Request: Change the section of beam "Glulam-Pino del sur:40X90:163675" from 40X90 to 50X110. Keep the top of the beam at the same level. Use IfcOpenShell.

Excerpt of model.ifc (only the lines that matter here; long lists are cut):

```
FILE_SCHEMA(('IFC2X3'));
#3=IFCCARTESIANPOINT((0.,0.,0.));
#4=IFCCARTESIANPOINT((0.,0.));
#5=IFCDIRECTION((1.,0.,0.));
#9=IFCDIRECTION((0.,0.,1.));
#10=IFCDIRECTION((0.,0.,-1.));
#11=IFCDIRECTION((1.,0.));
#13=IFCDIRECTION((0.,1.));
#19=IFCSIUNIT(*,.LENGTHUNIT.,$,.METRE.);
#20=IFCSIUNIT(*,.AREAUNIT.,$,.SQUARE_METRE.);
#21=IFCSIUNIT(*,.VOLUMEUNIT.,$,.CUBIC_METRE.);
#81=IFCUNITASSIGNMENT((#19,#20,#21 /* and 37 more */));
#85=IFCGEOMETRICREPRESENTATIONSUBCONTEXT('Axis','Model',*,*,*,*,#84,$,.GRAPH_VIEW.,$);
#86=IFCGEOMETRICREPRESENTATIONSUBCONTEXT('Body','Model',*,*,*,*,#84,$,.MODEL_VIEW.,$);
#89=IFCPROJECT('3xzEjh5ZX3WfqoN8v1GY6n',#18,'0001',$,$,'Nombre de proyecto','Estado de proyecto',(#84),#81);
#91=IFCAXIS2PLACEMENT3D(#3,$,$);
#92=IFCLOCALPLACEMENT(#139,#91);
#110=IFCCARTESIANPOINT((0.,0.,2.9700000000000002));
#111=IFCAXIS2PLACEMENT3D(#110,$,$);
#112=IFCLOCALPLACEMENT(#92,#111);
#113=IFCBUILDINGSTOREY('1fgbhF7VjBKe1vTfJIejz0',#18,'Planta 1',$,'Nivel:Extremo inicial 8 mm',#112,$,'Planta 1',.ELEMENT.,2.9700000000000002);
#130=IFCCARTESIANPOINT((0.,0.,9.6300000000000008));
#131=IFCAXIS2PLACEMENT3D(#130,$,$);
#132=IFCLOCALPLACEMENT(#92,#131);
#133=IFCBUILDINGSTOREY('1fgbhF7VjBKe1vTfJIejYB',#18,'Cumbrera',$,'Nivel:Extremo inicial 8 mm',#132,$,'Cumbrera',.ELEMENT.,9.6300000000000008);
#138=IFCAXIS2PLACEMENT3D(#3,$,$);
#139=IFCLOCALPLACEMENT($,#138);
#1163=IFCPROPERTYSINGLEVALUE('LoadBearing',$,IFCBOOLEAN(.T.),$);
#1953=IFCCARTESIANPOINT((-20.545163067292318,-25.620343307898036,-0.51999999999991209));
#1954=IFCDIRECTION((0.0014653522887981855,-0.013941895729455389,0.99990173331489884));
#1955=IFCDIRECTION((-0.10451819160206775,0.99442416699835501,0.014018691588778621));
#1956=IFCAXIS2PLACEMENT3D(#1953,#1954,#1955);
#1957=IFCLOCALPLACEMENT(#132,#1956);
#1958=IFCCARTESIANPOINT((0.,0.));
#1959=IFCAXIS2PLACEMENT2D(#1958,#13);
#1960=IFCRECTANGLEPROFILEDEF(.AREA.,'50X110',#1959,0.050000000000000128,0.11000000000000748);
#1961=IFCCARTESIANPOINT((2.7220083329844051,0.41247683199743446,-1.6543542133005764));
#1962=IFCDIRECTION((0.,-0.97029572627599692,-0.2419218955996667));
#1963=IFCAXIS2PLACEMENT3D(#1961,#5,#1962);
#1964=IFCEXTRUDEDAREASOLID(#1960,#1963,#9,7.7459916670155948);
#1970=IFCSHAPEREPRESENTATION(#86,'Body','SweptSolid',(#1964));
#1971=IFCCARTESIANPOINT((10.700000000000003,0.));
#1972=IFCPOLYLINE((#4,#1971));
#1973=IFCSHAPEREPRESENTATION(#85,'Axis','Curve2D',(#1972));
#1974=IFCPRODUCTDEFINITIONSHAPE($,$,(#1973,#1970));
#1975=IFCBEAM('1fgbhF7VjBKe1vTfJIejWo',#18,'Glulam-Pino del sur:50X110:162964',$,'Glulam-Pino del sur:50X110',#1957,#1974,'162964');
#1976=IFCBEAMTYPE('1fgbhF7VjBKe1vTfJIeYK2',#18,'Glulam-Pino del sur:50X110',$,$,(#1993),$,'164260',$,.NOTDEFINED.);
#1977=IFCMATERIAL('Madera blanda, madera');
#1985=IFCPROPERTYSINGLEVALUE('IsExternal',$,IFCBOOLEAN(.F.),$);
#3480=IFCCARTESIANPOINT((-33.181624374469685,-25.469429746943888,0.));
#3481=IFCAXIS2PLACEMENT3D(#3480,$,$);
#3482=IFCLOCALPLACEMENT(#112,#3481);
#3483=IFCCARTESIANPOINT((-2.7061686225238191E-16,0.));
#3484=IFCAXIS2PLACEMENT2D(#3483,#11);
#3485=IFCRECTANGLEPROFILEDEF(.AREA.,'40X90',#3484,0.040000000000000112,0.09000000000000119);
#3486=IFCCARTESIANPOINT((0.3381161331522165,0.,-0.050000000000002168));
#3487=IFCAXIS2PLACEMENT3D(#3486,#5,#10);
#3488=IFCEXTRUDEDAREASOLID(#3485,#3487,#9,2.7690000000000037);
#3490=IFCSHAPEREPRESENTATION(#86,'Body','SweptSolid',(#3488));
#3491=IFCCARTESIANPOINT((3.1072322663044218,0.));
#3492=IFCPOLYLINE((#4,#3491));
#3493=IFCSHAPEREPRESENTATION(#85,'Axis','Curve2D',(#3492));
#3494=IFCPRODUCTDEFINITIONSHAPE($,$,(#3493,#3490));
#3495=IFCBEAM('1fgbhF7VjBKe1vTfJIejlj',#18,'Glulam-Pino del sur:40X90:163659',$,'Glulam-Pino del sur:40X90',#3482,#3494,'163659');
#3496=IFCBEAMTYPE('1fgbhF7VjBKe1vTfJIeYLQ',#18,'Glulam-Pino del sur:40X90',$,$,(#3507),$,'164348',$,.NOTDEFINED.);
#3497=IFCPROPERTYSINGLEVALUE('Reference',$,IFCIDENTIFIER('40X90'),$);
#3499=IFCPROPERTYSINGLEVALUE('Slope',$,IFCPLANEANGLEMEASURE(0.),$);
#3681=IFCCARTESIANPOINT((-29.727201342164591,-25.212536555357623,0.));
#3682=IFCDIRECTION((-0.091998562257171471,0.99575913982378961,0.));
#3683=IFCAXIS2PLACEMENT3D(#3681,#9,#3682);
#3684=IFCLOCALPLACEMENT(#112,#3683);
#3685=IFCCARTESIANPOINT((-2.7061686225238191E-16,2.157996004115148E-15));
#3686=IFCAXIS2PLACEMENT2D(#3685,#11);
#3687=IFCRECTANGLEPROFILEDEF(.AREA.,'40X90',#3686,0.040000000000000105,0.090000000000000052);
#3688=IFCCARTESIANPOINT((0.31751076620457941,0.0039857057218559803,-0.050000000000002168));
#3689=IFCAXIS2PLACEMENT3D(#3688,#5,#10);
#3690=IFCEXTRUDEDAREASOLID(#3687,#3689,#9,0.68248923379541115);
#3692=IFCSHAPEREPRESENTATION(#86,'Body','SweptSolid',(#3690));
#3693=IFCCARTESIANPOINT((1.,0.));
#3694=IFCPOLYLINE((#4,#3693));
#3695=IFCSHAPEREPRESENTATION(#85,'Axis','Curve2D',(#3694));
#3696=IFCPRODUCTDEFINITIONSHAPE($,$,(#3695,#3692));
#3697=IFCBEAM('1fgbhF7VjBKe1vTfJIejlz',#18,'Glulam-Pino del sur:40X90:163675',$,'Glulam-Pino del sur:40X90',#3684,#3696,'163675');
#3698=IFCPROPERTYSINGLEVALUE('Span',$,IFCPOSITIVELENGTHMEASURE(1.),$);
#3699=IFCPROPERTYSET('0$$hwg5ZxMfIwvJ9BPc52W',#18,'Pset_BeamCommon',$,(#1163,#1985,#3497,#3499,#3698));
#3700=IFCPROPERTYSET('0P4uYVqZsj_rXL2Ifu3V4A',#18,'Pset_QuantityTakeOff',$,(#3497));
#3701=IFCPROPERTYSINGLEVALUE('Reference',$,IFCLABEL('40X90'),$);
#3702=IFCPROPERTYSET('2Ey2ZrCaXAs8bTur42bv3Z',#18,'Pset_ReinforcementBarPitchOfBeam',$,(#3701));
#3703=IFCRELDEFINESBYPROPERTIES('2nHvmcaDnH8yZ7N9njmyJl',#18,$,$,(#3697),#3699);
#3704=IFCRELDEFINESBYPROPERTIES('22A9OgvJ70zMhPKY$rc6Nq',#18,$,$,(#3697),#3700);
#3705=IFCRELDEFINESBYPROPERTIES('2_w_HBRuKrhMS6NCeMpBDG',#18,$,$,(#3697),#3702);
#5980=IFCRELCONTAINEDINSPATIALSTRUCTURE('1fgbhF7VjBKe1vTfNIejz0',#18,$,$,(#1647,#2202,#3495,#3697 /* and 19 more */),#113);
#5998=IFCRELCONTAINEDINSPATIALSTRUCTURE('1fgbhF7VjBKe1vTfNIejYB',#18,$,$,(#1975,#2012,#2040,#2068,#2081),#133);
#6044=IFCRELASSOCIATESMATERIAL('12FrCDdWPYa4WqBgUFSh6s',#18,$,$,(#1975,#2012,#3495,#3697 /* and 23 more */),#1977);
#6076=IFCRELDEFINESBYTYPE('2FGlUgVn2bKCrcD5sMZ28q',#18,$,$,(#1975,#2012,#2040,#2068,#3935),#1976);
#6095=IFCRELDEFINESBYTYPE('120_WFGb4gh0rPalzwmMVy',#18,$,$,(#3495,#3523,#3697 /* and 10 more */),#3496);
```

```python
import ifcopenshell
import ifcopenshell.api.pset
import ifcopenshell.api.type
import ifcopenshell.util.element
import ifcopenshell.util.representation

model = ifcopenshell.open("model.ifc")

member = model.by_guid("1fgbhF7VjBKe1vTfJIejlz")
source = next(p for p in model.by_type("IfcRectangleProfileDef") if p.ProfileName == "50X110")

body = ifcopenshell.util.representation.get_representation(member, "Model", "Body")
solid = body.Items[0]
old_profile = solid.SweptArea

# Copy the section's sizes but keep this member's own profile position.
profile = ifcopenshell.util.element.copy(model, source)
# Profiles are centred, so shift by half the change in depth to hold the top.
shift = (old_profile.XDim - profile.XDim) / 2
x, y = old_profile.Position.Location.Coordinates
up = (-1.0, 0.0)  # upwards, in the solid's own plane
location = model.createIfcCartesianPoint((x + up[0] * shift, y + up[1] * shift))
profile.Position = model.createIfcAxis2Placement2D(location, old_profile.Position.RefDirection)
solid.SweptArea = profile
if not model.get_total_inverses(old_profile):
    ifcopenshell.util.element.remove_deep2(model, old_profile)

new_type = model.by_id(1976)
ifcopenshell.api.type.assign_type(
    model, related_objects=[member], relating_type=new_type, should_map_representations=False
)
member.Name = member.Name.replace("40X90", "50X110")
member.ObjectType = "Glulam-Pino del sur:50X110"
pset = model.by_id(ifcopenshell.util.element.get_pset(member, "Pset_BeamCommon", should_inherit=False)["id"])
ifcopenshell.api.pset.edit_pset(model, pset=pset, properties={"Reference": "50X110"})
pset = model.by_id(ifcopenshell.util.element.get_pset(member, "Pset_QuantityTakeOff", should_inherit=False)["id"])
ifcopenshell.api.pset.edit_pset(model, pset=pset, properties={"Reference": "50X110"})
pset = model.by_id(ifcopenshell.util.element.get_pset(member, "Pset_ReinforcementBarPitchOfBeam", should_inherit=False)["id"])
ifcopenshell.api.pset.edit_pset(model, pset=pset, properties={"Reference": "50X110"})

print(solid.SweptArea)

model.write("model_rev.ifc")
```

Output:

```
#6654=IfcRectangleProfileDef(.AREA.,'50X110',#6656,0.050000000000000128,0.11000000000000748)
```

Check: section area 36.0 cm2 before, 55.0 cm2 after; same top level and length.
